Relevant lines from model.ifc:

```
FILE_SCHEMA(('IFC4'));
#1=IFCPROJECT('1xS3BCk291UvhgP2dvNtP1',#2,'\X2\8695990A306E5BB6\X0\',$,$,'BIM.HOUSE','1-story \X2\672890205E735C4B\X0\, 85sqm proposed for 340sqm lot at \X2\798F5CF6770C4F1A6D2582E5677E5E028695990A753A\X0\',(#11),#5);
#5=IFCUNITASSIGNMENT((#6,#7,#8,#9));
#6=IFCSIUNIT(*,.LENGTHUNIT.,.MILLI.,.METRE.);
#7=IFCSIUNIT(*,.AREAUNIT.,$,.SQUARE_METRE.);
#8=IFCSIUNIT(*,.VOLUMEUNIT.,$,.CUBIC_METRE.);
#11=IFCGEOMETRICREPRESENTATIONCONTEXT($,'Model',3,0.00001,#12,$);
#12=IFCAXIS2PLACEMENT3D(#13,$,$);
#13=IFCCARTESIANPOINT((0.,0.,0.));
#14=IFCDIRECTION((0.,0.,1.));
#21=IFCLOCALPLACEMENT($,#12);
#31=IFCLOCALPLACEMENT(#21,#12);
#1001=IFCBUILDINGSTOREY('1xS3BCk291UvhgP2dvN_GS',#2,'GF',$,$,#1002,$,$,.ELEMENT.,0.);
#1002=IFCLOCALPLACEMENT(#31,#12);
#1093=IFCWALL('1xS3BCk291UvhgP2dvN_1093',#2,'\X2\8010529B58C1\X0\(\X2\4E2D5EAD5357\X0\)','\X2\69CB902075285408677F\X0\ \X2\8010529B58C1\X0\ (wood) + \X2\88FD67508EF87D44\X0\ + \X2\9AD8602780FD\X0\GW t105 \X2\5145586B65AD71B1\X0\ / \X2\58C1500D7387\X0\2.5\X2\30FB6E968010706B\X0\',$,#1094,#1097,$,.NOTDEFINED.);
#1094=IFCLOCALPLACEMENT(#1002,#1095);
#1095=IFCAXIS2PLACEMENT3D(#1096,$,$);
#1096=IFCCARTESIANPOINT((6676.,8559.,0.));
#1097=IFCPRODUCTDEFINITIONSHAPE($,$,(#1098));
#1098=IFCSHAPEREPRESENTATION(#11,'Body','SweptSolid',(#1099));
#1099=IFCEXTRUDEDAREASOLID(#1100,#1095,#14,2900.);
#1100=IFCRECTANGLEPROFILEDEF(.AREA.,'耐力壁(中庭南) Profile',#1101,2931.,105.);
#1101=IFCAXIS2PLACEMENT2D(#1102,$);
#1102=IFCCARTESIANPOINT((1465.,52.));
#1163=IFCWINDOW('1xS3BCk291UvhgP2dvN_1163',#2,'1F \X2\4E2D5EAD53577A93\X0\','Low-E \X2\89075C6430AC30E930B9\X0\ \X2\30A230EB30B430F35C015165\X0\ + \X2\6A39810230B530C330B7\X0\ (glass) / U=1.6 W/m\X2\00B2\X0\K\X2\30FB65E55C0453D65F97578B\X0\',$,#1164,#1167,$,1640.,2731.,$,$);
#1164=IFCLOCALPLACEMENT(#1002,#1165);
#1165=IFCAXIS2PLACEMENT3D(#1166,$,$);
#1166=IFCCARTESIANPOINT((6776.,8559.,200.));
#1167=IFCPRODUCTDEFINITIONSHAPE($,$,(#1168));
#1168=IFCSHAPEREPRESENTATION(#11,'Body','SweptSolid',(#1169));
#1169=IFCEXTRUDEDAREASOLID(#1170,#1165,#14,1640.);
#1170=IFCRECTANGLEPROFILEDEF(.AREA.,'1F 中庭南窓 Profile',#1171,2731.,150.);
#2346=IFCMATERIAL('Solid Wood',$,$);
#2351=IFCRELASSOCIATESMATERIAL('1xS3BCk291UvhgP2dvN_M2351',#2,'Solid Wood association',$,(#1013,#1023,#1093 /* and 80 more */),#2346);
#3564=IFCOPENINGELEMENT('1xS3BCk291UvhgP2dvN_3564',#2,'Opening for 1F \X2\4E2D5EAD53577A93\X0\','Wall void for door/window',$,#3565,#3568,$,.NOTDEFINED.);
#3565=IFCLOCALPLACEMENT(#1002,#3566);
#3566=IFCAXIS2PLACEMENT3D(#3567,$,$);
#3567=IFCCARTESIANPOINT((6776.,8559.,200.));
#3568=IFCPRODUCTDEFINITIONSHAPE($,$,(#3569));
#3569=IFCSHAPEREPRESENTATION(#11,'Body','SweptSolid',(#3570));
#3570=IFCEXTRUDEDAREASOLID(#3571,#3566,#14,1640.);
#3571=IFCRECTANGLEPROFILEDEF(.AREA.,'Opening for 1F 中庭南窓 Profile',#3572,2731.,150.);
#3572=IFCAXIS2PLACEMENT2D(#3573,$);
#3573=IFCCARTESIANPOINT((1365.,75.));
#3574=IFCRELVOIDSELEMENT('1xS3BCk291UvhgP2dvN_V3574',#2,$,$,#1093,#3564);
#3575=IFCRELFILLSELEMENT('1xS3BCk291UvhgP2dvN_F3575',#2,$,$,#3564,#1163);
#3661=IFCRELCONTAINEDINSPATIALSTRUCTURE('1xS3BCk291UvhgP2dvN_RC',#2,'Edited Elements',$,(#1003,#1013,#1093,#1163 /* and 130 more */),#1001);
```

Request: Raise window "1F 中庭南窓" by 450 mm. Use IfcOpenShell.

```python
import numpy as np
import ifcopenshell
import ifcopenshell.api.geometry
import ifcopenshell.util.placement
import ifcopenshell.util.unit

model = ifcopenshell.open("model.ifc")
unit_scale = ifcopenshell.util.unit.calculate_unit_scale(model)

window = model.by_guid("1xS3BCk291UvhgP2dvN_1163")
opening = window.FillsVoids[0].RelatingOpeningElement
dz = 450.0

shift = np.array([0.0, 0.0, dz])
# The window is not placed relative to its opening, so move both.
for product in (opening, window):
    matrix = ifcopenshell.util.placement.get_local_placement(product.ObjectPlacement)
    matrix[:3, 3] += shift
    ifcopenshell.api.geometry.edit_object_placement(model, product=product, matrix=matrix, is_si=False)

print(f"moved by {dz * unit_scale:+.3f} m")

model.write("model-out.ifc")
```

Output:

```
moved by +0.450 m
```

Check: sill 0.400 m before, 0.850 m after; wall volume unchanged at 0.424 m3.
